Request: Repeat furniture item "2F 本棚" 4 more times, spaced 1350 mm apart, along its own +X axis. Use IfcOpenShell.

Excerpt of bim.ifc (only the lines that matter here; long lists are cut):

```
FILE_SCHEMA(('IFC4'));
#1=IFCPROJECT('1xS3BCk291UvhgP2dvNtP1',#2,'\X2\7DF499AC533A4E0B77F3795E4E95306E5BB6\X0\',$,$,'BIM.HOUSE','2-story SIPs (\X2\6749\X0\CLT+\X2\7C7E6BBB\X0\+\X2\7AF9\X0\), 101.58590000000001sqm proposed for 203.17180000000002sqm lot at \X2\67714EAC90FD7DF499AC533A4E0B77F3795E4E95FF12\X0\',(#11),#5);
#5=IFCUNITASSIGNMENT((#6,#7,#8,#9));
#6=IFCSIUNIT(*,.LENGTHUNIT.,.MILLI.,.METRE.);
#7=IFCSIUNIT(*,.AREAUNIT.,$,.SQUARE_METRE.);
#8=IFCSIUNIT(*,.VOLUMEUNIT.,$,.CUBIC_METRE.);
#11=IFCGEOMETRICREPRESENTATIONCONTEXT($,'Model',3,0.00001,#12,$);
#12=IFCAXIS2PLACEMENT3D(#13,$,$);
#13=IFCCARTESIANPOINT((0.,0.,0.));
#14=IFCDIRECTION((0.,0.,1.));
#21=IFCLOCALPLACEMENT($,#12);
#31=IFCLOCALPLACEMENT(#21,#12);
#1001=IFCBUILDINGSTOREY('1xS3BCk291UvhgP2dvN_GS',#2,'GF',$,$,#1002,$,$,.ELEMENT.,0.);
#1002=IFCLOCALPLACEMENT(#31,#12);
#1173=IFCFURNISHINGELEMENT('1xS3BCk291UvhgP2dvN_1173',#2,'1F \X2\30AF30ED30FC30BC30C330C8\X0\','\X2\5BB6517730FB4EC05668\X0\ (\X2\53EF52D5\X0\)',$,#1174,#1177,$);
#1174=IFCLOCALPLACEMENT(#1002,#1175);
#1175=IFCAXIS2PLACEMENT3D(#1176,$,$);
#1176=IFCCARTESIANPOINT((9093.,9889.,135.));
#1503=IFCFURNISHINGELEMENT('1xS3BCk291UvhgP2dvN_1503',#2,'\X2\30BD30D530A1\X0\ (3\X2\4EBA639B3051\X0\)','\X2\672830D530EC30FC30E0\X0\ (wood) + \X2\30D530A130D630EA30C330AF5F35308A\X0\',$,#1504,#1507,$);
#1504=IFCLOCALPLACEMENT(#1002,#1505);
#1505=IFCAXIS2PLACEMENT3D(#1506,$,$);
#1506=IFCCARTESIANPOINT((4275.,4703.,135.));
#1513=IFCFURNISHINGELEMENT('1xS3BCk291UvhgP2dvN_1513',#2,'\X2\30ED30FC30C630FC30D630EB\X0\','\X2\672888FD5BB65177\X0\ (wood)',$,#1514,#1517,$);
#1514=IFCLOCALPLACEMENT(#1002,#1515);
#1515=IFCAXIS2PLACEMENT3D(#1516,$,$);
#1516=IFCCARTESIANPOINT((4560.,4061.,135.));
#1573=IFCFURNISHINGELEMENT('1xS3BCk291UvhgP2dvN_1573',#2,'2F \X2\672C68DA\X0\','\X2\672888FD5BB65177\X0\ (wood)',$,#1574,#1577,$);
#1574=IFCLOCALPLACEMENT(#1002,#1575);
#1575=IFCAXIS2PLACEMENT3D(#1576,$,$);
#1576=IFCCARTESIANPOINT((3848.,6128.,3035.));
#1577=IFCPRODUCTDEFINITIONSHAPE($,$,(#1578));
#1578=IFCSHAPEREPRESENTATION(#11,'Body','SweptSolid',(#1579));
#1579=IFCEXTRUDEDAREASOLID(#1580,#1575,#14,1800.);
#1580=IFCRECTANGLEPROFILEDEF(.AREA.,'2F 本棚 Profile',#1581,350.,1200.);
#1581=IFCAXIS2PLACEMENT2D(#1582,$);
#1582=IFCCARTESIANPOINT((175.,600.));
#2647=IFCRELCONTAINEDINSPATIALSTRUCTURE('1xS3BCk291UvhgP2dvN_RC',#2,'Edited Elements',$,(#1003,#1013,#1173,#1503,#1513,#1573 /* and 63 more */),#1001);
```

```python
import ifcopenshell
import ifcopenshell.api.geometry
import ifcopenshell.api.root
import ifcopenshell.util.element
import ifcopenshell.util.placement
import ifcopenshell.util.unit

model = ifcopenshell.open("bim.ifc")
unit_scale = ifcopenshell.util.unit.calculate_unit_scale(model)


def reuse_history(source, copy):
    """copy_class also copies each property set's owner history, people and application; keep the originals."""
    for rel in copy.IsDefinedBy:
        if rel.is_a("IfcRelDefinesByProperties") and (history := rel.RelatingPropertyDefinition.OwnerHistory):
            rel.RelatingPropertyDefinition.OwnerHistory = source.OwnerHistory
            ifcopenshell.util.element.remove_deep2(model, history)


source = model.by_guid("1xS3BCk291UvhgP2dvN_1573")
base = ifcopenshell.util.placement.get_local_placement(source.ObjectPlacement)
step = base[:3, 0] * 1.35 / unit_scale

for i in range(1, 5):
    copy = ifcopenshell.api.root.copy_class(model, product=source)
    copy.Representation = ifcopenshell.util.element.copy_deep(
        model, source.Representation, exclude=["IfcGeometricRepresentationContext", "IfcRepresentationMap"]
    )
    reuse_history(source, copy)
    matrix = base.copy()
    matrix[:3, 3] += i * step
    print("added at", matrix[:3, 3].round(3) + 0.0)
    ifcopenshell.api.geometry.edit_object_placement(model, product=copy, matrix=matrix, is_si=False)

model.write("bim_v2.ifc")
```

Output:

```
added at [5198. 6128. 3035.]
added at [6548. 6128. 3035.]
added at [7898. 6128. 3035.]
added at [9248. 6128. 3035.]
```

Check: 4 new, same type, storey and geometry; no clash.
